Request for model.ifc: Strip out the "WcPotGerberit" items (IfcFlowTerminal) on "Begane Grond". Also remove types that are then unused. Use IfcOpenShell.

First a look at what the model holds.

```python
import ifcopenshell
import ifcopenshell.util.element

model = ifcopenshell.open("model.ifc")
print(model.schema)
storey = next(s for s in model.by_type("IfcBuildingStorey") if s.Name == "Begane Grond")
terminals = [e for e in ifcopenshell.util.element.get_decomposition(storey) if e.is_a("IfcFlowTerminal")]
seen = {}
for e in terminals:
    element_type = ifcopenshell.util.element.get_type(e)
    name = element_type.Name if element_type not in (None, e) else None
    seen[name] = seen.get(name, 0) + 1
for name, count in sorted(seen.items(), key=str):
    print(count, "x", name)
```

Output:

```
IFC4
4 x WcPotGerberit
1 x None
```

```python
import ifcopenshell
import ifcopenshell.api.root
import ifcopenshell.util.element

model = ifcopenshell.open("model.ifc")

storey = next(s for s in model.by_type("IfcBuildingStorey") if s.Name == "Begane Grond")
terminals = [e for e in ifcopenshell.util.element.get_decomposition(storey) if e.is_a("IfcFlowTerminal")]
targets = [e for e in terminals if (t := ifcopenshell.util.element.get_type(e)) not in (None, e) and t.Name == "WcPotGerberit"]
types = {ifcopenshell.util.element.get_type(e) for e in targets} - {None, *targets}

for e in targets:
    ifcopenshell.api.root.remove_product(model, product=e)
print(len(targets), "removed")

unused = [t for t in types if not ifcopenshell.util.element.get_types(t)]
for t in unused:
    ifcopenshell.api.root.remove_product(model, product=t)
print(len(unused), "unused types removed")

model.write("model_edited.ifc")
```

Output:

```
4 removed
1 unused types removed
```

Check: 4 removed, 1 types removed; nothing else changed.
